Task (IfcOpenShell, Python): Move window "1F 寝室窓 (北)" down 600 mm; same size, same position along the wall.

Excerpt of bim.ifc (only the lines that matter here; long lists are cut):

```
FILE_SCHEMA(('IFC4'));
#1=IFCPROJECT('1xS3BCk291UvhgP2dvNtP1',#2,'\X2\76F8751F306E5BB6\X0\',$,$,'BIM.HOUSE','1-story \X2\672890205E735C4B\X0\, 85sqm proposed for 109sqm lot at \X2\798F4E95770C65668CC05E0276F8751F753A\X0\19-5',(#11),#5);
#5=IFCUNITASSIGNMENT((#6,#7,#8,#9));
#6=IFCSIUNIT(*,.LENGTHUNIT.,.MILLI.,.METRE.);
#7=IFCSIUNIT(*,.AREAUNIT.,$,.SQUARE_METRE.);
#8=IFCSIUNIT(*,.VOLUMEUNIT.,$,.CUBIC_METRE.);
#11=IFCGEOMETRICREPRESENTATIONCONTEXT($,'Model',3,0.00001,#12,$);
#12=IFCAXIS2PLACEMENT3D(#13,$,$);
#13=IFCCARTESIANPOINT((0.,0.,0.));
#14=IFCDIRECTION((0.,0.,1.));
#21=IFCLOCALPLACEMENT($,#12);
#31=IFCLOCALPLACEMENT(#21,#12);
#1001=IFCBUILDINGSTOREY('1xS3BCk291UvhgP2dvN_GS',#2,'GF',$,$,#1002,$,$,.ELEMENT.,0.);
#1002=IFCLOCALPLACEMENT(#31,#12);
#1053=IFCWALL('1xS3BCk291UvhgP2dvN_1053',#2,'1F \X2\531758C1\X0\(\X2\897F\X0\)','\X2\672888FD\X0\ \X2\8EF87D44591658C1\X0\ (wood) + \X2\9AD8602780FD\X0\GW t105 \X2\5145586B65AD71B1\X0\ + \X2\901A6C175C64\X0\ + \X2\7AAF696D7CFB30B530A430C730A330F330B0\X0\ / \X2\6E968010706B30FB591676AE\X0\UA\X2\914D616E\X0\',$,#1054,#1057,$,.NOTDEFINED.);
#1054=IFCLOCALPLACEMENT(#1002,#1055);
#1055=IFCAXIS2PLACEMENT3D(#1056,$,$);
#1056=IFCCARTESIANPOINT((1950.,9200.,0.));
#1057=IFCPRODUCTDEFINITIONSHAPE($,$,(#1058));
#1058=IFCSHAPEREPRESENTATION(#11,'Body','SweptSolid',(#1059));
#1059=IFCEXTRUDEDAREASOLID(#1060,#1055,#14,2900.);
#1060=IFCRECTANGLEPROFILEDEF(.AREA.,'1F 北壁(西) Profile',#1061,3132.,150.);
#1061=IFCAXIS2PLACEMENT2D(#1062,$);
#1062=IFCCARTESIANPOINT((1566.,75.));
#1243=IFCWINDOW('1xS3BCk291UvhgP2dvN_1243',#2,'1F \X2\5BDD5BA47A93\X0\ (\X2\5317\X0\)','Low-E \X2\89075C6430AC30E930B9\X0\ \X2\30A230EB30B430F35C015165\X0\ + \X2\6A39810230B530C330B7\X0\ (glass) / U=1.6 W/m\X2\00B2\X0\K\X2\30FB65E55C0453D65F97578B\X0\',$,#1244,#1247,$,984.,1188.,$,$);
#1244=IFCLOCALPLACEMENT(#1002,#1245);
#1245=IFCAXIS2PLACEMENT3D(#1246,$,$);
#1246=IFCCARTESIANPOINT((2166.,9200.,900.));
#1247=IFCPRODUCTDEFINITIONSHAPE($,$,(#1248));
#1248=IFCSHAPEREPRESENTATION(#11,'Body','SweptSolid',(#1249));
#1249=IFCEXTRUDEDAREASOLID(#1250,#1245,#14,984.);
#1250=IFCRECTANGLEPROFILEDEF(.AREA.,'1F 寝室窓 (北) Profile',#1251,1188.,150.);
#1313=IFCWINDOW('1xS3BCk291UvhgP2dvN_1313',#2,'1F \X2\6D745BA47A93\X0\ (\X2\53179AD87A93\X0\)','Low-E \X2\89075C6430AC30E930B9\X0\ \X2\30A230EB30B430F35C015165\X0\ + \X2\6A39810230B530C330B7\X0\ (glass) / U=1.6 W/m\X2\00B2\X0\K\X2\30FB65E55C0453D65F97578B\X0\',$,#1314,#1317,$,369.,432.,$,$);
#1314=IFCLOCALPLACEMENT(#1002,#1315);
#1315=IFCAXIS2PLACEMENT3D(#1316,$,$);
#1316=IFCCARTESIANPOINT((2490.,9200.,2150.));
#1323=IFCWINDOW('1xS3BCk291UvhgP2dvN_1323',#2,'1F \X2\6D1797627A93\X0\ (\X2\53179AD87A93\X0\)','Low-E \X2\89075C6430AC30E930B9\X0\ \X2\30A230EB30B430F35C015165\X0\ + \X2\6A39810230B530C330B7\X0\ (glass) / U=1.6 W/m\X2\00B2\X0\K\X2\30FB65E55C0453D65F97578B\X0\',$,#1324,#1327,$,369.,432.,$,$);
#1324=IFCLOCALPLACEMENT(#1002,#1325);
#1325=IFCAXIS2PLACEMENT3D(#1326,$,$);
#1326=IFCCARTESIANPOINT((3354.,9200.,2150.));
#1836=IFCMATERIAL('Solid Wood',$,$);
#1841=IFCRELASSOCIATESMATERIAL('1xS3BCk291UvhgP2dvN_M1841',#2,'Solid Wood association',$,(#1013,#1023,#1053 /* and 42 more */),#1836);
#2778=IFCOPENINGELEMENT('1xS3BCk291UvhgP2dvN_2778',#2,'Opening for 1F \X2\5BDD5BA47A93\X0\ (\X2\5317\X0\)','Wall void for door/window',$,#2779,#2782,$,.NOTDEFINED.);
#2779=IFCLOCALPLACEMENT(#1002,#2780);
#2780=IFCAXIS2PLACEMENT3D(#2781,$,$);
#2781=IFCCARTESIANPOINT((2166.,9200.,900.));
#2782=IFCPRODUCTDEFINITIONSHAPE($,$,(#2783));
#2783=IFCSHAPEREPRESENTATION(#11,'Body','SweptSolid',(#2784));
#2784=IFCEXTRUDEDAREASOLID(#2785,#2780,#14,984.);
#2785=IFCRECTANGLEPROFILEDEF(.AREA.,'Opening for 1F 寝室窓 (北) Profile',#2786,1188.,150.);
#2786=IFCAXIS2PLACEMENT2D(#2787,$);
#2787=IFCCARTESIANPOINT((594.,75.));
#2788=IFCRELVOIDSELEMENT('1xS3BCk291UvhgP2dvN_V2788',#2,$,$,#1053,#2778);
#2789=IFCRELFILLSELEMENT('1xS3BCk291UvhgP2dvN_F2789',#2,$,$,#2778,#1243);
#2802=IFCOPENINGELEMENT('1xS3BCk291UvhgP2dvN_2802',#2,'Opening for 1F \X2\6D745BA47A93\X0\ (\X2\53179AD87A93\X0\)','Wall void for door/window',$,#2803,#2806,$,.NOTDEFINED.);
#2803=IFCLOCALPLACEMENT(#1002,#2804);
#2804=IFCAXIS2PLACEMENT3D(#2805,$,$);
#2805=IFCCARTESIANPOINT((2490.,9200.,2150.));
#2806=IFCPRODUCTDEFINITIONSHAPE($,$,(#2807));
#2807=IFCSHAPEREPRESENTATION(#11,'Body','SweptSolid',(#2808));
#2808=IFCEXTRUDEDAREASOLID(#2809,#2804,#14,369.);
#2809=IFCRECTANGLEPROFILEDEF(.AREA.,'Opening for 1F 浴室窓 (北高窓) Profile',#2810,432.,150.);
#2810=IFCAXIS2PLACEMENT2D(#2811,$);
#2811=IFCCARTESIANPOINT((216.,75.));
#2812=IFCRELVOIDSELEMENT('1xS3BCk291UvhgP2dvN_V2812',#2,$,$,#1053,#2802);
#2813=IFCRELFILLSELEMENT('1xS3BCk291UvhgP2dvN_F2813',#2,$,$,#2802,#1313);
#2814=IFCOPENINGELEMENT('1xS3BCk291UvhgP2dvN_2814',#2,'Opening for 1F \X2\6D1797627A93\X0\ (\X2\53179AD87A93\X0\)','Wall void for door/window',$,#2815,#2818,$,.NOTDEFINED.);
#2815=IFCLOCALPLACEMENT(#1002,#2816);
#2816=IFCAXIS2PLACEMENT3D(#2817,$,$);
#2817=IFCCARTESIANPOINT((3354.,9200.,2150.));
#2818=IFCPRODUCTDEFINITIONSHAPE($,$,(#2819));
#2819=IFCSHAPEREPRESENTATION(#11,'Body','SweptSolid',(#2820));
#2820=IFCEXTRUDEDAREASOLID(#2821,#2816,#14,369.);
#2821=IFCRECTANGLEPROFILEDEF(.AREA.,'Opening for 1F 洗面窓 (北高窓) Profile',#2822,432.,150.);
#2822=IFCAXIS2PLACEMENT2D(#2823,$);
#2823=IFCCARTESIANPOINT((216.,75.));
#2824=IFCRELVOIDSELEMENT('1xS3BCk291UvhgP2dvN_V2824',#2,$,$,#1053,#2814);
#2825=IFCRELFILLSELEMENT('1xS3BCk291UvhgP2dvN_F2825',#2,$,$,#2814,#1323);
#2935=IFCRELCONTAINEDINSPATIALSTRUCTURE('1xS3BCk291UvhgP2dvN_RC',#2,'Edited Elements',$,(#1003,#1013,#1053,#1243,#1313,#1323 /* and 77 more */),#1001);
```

```python
import numpy as np
import ifcopenshell
import ifcopenshell.api.geometry
import ifcopenshell.util.placement
import ifcopenshell.util.unit

model = ifcopenshell.open("bim.ifc")
unit_scale = ifcopenshell.util.unit.calculate_unit_scale(model)

window = model.by_id(1243)
opening = window.FillsVoids[0].RelatingOpeningElement
dz = -600.0

shift = np.array([0.0, 0.0, dz])
# The window is not placed relative to its opening, so move both.
for product in (opening, window):
    matrix = ifcopenshell.util.placement.get_local_placement(product.ObjectPlacement)
    matrix[:3, 3] += shift
    ifcopenshell.api.geometry.edit_object_placement(model, product=product, matrix=matrix, is_si=False)

print(f"moved by {dz * unit_scale:+.3f} m")

model.write("bim_updated.ifc")
```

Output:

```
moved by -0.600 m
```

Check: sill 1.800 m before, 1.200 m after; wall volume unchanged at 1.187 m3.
